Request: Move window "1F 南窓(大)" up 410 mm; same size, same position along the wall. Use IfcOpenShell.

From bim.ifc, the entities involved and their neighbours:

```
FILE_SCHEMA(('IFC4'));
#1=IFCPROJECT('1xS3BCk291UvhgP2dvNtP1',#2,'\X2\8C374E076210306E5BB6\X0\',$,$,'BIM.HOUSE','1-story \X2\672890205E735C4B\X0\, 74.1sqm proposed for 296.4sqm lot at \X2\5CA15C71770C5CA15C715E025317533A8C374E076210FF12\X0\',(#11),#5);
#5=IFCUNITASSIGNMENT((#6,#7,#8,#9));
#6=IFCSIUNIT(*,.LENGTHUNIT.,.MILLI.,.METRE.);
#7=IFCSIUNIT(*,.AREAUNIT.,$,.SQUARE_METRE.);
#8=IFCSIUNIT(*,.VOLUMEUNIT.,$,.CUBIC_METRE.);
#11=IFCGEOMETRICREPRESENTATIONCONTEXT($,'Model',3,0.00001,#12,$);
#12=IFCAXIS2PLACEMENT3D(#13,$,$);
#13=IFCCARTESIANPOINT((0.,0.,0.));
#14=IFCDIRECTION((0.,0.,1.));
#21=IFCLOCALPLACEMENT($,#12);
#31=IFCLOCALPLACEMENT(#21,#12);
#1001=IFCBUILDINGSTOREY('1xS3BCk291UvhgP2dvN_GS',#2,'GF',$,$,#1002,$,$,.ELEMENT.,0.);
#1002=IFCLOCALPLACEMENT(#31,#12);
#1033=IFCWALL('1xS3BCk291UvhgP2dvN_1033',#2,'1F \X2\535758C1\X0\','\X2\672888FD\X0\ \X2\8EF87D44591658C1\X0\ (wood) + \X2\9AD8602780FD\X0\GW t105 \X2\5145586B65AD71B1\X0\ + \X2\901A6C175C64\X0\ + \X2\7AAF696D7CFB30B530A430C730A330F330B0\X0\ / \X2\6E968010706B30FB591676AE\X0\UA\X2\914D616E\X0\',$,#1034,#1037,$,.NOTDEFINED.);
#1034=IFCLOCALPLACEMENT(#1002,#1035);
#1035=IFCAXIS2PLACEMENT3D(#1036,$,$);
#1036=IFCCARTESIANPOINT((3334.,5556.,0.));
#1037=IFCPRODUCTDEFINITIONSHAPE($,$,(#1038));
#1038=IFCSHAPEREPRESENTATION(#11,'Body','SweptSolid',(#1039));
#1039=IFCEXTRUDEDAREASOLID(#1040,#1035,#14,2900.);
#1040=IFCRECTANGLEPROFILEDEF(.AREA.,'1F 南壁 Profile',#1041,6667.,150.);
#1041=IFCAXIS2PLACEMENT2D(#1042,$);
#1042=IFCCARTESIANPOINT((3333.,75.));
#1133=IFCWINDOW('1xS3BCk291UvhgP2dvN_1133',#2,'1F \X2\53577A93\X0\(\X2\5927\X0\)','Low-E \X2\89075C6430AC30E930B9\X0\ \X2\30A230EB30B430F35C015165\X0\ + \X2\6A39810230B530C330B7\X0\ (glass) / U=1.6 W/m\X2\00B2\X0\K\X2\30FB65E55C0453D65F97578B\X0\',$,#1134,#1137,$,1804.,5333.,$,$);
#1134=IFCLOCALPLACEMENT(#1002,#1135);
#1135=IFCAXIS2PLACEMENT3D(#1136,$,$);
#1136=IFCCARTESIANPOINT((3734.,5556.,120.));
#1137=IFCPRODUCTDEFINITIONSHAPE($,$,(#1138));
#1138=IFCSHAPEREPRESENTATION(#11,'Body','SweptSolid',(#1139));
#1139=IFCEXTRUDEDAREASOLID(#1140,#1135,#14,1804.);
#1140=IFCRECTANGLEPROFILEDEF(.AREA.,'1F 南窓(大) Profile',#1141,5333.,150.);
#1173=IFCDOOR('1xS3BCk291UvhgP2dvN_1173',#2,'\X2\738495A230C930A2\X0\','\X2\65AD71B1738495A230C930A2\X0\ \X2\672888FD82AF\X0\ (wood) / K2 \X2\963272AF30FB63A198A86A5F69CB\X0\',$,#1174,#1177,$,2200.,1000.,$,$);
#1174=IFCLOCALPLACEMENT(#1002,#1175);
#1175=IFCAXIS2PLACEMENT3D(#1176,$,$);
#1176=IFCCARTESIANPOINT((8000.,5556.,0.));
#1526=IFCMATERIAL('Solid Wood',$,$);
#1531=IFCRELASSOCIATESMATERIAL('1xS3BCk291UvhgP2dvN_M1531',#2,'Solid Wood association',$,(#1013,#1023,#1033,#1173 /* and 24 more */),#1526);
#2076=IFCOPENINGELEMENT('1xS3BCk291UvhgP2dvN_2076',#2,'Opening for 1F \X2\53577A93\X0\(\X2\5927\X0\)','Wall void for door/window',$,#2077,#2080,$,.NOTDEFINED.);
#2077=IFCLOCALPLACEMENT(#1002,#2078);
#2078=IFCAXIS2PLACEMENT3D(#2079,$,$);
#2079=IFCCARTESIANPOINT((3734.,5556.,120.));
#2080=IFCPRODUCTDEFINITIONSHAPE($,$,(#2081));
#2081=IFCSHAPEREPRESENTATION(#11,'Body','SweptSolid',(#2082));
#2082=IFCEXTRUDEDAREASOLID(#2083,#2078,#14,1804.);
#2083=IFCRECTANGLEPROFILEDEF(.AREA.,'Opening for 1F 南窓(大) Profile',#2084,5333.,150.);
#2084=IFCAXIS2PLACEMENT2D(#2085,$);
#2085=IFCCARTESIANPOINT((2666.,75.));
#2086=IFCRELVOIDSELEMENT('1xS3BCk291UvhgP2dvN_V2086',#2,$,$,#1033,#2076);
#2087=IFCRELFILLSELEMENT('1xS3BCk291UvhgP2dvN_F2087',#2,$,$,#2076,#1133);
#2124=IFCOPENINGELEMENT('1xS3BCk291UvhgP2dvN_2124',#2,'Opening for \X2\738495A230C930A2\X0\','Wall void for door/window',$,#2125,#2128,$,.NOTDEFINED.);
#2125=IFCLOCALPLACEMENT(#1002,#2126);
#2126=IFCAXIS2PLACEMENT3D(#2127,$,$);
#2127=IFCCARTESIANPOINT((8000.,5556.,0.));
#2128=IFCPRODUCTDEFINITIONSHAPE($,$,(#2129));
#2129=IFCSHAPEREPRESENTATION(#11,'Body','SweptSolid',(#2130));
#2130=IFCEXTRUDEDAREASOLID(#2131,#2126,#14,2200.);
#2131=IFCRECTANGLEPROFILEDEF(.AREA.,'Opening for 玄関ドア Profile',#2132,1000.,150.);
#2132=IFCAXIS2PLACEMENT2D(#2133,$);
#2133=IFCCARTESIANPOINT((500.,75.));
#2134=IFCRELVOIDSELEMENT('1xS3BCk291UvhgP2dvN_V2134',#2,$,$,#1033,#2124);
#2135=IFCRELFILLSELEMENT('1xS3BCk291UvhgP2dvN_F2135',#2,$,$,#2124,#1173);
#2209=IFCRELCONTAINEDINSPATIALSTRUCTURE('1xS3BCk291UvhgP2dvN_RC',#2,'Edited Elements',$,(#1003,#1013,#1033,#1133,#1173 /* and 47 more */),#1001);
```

```python
import numpy as np
import ifcopenshell
import ifcopenshell.api.geometry
import ifcopenshell.util.placement
import ifcopenshell.util.unit

model = ifcopenshell.open("bim.ifc")
unit_scale = ifcopenshell.util.unit.calculate_unit_scale(model)

window = model.by_guid("1xS3BCk291UvhgP2dvN_1133")
opening = window.FillsVoids[0].RelatingOpeningElement
dz = 410.0

shift = np.array([0.0, 0.0, dz])
# The window is not placed relative to its opening, so move both.
for product in (opening, window):
    matrix = ifcopenshell.util.placement.get_local_placement(product.ObjectPlacement)
    matrix[:3, 3] += shift
    ifcopenshell.api.geometry.edit_object_placement(model, product=product, matrix=matrix, is_si=False)

print(f"moved by {dz * unit_scale:+.3f} m")

model.write("bim_rev.ifc")
```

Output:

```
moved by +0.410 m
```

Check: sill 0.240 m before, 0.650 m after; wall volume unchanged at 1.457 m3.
